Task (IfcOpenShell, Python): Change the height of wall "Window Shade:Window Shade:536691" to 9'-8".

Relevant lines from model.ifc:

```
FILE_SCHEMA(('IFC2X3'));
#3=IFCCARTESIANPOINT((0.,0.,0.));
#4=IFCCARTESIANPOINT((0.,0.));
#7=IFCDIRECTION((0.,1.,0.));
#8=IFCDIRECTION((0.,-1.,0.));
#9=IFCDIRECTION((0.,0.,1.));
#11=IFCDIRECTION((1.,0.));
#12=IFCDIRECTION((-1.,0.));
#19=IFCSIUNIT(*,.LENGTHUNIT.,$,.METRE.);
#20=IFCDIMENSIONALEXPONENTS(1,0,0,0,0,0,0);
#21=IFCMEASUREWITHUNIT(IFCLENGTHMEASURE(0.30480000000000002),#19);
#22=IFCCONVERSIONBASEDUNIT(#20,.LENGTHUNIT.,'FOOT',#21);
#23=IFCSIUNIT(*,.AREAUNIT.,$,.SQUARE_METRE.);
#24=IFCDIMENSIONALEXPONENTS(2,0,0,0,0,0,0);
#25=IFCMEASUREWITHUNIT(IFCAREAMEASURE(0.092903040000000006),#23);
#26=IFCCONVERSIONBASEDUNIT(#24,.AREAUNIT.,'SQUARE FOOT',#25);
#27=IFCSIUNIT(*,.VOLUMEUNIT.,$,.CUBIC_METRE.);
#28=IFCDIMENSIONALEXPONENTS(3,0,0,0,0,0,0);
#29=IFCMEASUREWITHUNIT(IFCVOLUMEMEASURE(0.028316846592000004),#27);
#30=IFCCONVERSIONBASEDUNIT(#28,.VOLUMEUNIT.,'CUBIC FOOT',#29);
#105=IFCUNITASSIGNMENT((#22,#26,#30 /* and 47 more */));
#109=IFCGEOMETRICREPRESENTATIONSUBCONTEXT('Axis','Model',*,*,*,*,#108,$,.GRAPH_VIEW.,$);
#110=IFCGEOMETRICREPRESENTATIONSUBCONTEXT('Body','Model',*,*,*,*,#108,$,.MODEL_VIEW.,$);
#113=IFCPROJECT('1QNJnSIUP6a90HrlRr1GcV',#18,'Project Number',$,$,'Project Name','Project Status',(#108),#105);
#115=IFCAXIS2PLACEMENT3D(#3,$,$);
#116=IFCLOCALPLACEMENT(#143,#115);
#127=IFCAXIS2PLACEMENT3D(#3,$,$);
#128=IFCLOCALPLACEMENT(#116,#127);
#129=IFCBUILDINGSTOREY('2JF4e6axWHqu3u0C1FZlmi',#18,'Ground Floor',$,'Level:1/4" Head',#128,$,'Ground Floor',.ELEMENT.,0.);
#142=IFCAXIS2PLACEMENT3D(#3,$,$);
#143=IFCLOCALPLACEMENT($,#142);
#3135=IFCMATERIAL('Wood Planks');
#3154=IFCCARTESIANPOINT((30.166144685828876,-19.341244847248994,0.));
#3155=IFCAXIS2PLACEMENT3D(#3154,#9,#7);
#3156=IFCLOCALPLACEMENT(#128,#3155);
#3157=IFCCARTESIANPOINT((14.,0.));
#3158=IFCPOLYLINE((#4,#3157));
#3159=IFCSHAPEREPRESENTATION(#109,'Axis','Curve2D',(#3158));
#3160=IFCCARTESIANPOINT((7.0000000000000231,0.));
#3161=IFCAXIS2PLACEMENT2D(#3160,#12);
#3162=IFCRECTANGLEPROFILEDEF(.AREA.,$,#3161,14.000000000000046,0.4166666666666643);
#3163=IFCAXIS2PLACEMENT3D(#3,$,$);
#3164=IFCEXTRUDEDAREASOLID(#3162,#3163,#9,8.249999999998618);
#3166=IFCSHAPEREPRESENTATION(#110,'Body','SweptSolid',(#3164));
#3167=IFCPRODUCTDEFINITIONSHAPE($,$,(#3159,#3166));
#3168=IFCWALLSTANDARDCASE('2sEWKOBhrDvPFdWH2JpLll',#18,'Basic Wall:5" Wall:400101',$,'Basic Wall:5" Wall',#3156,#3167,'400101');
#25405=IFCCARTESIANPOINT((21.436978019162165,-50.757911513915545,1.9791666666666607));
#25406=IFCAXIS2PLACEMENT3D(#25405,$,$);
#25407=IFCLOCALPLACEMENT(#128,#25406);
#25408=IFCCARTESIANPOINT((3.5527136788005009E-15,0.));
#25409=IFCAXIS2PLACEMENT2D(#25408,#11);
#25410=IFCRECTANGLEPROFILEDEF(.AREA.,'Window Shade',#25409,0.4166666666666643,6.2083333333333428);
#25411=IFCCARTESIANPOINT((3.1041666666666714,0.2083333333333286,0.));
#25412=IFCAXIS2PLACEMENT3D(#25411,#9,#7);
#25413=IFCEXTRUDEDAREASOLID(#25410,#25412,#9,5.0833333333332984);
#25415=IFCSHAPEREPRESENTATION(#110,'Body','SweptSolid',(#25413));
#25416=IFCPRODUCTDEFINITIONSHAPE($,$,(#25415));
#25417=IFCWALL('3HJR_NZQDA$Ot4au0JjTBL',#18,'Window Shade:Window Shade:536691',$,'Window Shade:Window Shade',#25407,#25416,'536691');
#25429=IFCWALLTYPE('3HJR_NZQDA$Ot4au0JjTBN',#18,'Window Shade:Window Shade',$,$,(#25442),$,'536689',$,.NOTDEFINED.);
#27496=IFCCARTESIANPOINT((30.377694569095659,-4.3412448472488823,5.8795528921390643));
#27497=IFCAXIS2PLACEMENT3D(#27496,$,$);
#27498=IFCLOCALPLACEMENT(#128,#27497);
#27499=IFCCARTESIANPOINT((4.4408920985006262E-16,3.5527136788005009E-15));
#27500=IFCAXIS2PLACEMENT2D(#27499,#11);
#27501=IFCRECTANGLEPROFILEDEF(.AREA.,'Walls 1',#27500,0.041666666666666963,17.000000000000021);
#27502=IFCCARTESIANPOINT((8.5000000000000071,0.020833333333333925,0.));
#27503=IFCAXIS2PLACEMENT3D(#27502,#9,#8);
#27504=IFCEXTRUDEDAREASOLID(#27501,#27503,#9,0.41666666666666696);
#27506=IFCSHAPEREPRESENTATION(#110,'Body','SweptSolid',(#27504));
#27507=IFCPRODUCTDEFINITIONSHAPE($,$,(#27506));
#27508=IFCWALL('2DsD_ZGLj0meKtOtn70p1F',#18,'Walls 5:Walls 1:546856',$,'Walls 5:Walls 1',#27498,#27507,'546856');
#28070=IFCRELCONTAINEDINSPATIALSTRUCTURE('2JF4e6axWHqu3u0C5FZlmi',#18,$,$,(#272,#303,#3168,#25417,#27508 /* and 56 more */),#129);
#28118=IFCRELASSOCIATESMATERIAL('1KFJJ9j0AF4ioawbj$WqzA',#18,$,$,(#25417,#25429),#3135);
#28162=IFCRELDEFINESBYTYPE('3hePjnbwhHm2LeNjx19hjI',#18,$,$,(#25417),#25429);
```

```python
import ifcopenshell
import ifcopenshell.geom
import ifcopenshell.util.representation
import ifcopenshell.util.shape
import ifcopenshell.util.unit

model = ifcopenshell.open("model.ifc")
unit_scale = ifcopenshell.util.unit.calculate_unit_scale(model)
settings = ifcopenshell.geom.settings()


def volume(element):
    """Net volume in cubic metres, openings subtracted."""
    shape = ifcopenshell.geom.create_shape(settings, element)
    return ifcopenshell.util.shape.get_volume(shape.geometry)


wall = model.by_guid("3HJR_NZQDA$Ot4au0JjTBL")
before = volume(wall)

body = ifcopenshell.util.representation.get_representation(wall, "Model", "Body")
solid = body.Items[0]
old_height = solid.Depth
solid.Depth = 116 * 0.0254 / unit_scale
after = volume(wall)

print(f"height {old_height:g} -> {solid.Depth:g}, volume {before:.3f} -> {after:.3f} m3")

model.write("model-out.ifc")
```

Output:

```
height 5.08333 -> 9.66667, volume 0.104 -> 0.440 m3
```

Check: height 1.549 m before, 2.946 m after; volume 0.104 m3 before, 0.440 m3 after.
